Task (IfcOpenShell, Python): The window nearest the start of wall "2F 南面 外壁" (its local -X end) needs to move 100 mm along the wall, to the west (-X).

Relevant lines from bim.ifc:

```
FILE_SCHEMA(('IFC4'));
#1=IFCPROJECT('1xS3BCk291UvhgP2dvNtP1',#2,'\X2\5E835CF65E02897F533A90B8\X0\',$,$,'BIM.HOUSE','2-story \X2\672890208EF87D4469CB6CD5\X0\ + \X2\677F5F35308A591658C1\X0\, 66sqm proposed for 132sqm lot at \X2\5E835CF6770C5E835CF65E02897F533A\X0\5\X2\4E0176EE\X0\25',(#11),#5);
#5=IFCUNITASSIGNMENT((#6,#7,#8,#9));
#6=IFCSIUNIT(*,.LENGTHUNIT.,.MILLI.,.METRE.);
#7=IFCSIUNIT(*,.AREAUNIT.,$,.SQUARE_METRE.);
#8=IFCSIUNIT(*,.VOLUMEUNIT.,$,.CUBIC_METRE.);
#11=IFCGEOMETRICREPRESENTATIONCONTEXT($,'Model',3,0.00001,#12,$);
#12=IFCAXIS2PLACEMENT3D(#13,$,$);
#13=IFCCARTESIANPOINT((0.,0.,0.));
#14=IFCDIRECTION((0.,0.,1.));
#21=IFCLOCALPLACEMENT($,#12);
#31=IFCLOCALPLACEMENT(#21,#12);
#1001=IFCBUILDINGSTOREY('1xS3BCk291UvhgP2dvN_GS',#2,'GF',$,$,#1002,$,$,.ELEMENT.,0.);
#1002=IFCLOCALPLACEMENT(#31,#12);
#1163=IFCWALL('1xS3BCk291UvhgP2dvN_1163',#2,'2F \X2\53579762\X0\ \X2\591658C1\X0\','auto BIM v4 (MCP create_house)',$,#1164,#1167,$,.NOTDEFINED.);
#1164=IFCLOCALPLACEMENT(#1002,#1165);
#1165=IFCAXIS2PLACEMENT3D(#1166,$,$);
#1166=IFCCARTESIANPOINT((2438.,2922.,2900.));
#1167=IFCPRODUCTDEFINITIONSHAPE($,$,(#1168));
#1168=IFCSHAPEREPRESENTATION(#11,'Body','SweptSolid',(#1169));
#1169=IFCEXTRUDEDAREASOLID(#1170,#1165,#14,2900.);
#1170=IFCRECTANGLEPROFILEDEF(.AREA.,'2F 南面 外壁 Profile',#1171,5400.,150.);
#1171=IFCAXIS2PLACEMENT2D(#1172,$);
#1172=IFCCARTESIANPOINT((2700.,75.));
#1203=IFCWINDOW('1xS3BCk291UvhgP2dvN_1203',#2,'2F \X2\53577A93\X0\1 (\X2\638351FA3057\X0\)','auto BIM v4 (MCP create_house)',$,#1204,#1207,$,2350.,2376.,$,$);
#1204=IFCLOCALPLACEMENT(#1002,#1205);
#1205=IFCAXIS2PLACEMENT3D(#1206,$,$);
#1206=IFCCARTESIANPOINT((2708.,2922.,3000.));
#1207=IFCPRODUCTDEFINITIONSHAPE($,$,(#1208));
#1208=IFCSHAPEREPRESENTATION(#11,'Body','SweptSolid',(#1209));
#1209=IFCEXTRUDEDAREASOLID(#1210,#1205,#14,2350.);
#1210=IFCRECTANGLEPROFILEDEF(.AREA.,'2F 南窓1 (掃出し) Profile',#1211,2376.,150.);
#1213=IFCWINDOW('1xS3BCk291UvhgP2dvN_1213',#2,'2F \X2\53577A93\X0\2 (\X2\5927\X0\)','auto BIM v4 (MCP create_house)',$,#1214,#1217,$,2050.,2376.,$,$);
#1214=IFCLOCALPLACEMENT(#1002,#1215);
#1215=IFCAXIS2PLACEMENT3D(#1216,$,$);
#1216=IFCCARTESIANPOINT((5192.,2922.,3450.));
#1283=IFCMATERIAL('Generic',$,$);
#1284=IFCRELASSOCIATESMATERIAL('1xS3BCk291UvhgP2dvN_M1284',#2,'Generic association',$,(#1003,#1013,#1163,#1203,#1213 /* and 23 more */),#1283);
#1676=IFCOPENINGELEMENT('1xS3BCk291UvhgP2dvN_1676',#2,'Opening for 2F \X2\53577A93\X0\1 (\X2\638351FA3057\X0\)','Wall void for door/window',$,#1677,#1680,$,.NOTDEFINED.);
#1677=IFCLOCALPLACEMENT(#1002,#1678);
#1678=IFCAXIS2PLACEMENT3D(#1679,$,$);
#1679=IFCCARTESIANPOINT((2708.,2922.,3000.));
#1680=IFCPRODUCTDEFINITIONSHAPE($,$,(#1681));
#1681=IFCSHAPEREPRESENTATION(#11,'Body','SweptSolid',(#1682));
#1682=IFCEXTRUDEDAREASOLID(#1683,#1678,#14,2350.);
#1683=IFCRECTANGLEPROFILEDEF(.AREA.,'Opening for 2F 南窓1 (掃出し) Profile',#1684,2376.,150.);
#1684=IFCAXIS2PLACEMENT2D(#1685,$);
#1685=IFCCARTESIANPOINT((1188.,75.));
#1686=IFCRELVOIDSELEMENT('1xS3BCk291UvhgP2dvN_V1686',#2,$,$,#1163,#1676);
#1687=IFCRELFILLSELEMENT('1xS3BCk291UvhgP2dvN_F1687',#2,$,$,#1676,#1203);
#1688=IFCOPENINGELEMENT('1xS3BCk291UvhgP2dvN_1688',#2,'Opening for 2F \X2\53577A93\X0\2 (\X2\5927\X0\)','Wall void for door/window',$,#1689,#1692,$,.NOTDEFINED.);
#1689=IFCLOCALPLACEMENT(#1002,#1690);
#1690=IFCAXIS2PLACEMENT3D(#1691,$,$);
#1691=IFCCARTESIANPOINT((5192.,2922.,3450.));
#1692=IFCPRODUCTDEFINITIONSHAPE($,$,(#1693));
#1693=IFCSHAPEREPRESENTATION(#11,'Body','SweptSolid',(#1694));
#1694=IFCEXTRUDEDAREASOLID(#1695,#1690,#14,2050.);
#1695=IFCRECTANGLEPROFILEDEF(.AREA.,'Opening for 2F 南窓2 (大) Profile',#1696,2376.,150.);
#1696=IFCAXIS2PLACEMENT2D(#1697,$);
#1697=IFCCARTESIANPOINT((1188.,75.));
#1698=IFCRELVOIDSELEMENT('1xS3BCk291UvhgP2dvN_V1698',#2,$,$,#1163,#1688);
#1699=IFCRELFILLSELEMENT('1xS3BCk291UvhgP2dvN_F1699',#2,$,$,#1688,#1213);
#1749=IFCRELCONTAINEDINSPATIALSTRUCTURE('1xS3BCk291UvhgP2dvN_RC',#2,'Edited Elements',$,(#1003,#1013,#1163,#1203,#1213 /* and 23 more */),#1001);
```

```python
import ifcopenshell
import ifcopenshell.api.geometry
import ifcopenshell.util.placement

model = ifcopenshell.open("bim.ifc")

window = model.by_guid("1xS3BCk291UvhgP2dvN_1203")
opening = window.FillsVoids[0].RelatingOpeningElement
wall = opening.VoidsElements[0].RelatingBuildingElement

wall_matrix = ifcopenshell.util.placement.get_local_placement(wall.ObjectPlacement)
shift = wall_matrix[:3, 0] * -100.0
before = ifcopenshell.util.placement.get_local_placement(window.ObjectPlacement)[:3, 3].copy()

# The window is not placed relative to its opening, so move both.
for product in (opening, window):
    matrix = ifcopenshell.util.placement.get_local_placement(product.ObjectPlacement)
    matrix[:3, 3] += shift
    ifcopenshell.api.geometry.edit_object_placement(model, product=product, matrix=matrix, is_si=False)

after = ifcopenshell.util.placement.get_local_placement(window.ObjectPlacement)[:3, 3]
print("window moved by", (after - before).round(3) + 0.0)

model.write("bim_updated.ifc")
```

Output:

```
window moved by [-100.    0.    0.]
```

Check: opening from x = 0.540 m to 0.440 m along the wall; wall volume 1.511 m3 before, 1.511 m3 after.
